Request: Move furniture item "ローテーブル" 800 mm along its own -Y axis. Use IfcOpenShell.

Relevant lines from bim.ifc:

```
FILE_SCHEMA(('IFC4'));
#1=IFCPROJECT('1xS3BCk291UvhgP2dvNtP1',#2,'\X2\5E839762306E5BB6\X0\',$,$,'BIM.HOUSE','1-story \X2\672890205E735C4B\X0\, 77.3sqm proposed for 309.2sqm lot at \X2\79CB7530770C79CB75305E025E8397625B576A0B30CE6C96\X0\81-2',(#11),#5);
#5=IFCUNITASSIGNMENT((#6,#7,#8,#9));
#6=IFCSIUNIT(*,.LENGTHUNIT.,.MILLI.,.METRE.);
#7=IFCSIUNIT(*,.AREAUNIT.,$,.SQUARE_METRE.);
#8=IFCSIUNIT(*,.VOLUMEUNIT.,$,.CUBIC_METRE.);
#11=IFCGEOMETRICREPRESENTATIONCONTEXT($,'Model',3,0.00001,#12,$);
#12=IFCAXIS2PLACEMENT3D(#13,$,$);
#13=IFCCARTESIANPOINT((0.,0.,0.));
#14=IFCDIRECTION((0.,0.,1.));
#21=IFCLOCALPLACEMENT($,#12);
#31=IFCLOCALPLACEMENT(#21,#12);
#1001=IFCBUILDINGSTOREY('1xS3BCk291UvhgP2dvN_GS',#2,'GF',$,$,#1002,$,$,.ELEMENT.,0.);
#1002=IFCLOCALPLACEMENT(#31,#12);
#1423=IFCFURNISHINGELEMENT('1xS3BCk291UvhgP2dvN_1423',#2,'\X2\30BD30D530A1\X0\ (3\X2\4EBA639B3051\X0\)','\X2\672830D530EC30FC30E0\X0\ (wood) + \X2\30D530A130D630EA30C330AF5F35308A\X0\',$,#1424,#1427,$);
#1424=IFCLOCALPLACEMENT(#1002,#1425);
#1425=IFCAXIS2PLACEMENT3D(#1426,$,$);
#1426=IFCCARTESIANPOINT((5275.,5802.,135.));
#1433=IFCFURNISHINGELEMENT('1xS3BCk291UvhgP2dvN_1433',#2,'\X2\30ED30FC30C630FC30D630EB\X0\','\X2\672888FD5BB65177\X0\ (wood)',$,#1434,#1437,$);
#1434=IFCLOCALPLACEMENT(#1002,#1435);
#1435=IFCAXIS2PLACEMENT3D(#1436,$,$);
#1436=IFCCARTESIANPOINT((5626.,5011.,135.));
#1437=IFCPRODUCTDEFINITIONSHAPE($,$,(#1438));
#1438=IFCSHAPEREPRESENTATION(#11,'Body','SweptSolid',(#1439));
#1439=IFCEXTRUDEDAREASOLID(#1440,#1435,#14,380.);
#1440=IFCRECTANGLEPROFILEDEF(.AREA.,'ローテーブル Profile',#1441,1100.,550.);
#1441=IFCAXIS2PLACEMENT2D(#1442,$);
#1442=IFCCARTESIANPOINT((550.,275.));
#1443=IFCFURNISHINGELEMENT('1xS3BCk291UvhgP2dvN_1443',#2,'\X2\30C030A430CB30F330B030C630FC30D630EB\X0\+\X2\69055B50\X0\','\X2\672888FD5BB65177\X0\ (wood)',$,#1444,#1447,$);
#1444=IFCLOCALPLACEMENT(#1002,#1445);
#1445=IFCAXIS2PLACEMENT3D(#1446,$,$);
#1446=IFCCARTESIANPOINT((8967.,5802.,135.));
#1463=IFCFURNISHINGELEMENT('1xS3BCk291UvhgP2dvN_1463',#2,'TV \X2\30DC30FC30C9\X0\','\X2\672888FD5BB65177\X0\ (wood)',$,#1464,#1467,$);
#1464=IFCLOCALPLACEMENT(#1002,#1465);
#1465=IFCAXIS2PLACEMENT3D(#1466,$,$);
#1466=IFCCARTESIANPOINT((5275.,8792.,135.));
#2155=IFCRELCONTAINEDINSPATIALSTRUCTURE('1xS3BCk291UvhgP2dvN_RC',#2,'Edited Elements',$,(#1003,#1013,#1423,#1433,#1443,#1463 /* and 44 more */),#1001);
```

```python
import ifcopenshell
import ifcopenshell.api.geometry
import ifcopenshell.util.placement
import ifcopenshell.util.unit

model = ifcopenshell.open("bim.ifc")
unit_scale = ifcopenshell.util.unit.calculate_unit_scale(model)

item = model.by_guid("1xS3BCk291UvhgP2dvN_1433")
matrix = ifcopenshell.util.placement.get_local_placement(item.ObjectPlacement)
matrix[:3, 3] -= matrix[:3, 1] * 0.8 / unit_scale
ifcopenshell.api.geometry.edit_object_placement(model, product=item, matrix=matrix, is_si=False)

print(ifcopenshell.util.placement.get_local_placement(item.ObjectPlacement).round(3) + 0.0)

model.write("bim_v2.ifc")
```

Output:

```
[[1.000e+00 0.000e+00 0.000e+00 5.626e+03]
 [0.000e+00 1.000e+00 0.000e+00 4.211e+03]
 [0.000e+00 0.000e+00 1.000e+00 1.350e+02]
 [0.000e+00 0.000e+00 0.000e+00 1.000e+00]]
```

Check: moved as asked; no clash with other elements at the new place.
